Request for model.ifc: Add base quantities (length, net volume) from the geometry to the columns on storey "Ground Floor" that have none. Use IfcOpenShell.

First a look at what the model holds.

```python
import ifcopenshell
import ifcopenshell.util.element
import ifcopenshell.util.unit

model = ifcopenshell.open("model.ifc")
print(model.schema)
for unit_type in ("LENGTHUNIT", "AREAUNIT", "VOLUMEUNIT"):
    print(unit_type, ifcopenshell.util.unit.calculate_unit_scale(model, unit_type))
storey = next(s for s in model.by_type("IfcBuildingStorey") if s.Name == "Ground Floor")
columns = [e for e in ifcopenshell.util.element.get_decomposition(storey) if e.is_a("IfcColumn")]
for e in sorted(columns, key=lambda e: e.id()):
    print(e.id(), e.is_a(), e.Name, list(ifcopenshell.util.element.get_psets(e, qtos_only=True)), sep=" | ")
```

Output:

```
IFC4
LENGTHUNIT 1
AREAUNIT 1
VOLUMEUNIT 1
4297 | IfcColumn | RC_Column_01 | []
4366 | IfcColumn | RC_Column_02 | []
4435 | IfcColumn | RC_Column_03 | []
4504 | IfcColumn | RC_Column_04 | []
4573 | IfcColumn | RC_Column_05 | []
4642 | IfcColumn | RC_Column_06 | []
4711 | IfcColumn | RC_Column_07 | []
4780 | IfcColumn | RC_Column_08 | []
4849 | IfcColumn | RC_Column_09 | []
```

```python
import ifcopenshell
import ifcopenshell.api.pset
import ifcopenshell.geom
import ifcopenshell.util.element
import ifcopenshell.util.shape
import ifcopenshell.util.unit

model = ifcopenshell.open("model.ifc")
unit_scale = ifcopenshell.util.unit.calculate_unit_scale(model)
volume_scale = ifcopenshell.util.unit.calculate_unit_scale(model, "VOLUMEUNIT")
settings = ifcopenshell.geom.settings()

storey = next(s for s in model.by_type("IfcBuildingStorey") if s.Name == "Ground Floor")
columns = [e for e in ifcopenshell.util.element.get_decomposition(storey) if e.is_a("IfcColumn")]

for e in sorted(columns, key=lambda e: e.id()):
    if ifcopenshell.util.element.get_psets(e, qtos_only=True, should_inherit=False):
        continue
    # Geometry comes back in metres, in the element's own axes.
    shape = ifcopenshell.geom.create_shape(settings, e)
    values = {
        "Length": ifcopenshell.util.shape.get_z(shape.geometry) / unit_scale,
        "NetVolume": ifcopenshell.util.shape.get_volume(shape.geometry) / volume_scale,
    }
    qto = ifcopenshell.api.pset.add_qto(model, product=e, name="Qto_ColumnBaseQuantities")
    ifcopenshell.api.pset.edit_qto(model, qto=qto, properties=values)
    print(e.id(), {k: round(v, 3) for k, v in values.items()})

model.write("model_edited.ifc")
```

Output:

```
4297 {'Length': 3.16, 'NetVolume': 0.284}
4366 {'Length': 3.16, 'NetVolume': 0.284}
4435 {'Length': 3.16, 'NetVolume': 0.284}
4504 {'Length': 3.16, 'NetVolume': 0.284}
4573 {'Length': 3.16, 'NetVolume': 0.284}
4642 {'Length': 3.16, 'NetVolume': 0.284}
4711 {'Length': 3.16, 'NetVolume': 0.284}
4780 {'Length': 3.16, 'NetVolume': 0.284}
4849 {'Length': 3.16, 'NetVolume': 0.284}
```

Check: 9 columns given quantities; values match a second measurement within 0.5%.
